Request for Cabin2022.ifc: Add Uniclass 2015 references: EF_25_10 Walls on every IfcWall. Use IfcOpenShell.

First a look at what the model holds.

```python
import ifcopenshell

model = ifcopenshell.open("Cabin2022.ifc")
print(model.schema)
print("classifications:", [c.Name for c in model.by_type("IfcClassification")])
for ifc_class in ("IfcDoor", "IfcRoof", "IfcStair", "IfcWall", "IfcWindow"):
    print(ifc_class, len(model.by_type(ifc_class)))
```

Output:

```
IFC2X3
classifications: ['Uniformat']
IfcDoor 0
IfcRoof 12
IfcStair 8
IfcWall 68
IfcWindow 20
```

```python
import ifcopenshell
import ifcopenshell.api.classification

model = ifcopenshell.open("Cabin2022.ifc")

# IFC2X3 requires Source and Edition and has no link from the project to the system.
system = model.create_entity("IfcClassification", Source="NBS", Edition="2015", Name="Uniclass 2015")

codes = {
    "IfcWall": ("EF_25_10", "Walls"),
}
for ifc_class, (code, name) in codes.items():
    products = model.by_type(ifc_class)
    ifcopenshell.api.classification.add_reference(
        model, products=products, classification=system, identification=code, name=name
    )
    print(code, len(products))

model.write("Cabin2022_rev.ifc")
```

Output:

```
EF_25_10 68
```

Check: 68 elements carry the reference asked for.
